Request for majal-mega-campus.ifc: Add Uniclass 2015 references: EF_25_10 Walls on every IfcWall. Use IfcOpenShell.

First a look at what the model holds.

```python
import ifcopenshell

model = ifcopenshell.open("majal-mega-campus.ifc")
print(model.schema)
print("classifications:", [c.Name for c in model.by_type("IfcClassification")])
for ifc_class in ("IfcDoor", "IfcRoof", "IfcStair", "IfcWall", "IfcWindow"):
    print(ifc_class, len(model.by_type(ifc_class)))
```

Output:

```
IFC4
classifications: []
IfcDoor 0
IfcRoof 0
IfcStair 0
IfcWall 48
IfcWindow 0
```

```python
import ifcopenshell
import ifcopenshell.api.classification

model = ifcopenshell.open("majal-mega-campus.ifc")

system = ifcopenshell.api.classification.add_classification(model, classification="Uniclass 2015")

codes = {
    "IfcWall": ("EF_25_10", "Walls"),
}
for ifc_class, (code, name) in codes.items():
    products = model.by_type(ifc_class)
    ifcopenshell.api.classification.add_reference(
        model, products=products, classification=system, identification=code, name=name
    )
    print(code, len(products))

model.write("majal-mega-campus_v2.ifc")
```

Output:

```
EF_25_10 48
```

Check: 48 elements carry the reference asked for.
